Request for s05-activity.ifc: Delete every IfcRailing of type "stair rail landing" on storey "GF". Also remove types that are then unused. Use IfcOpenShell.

First a look at what the model holds.

```python
import ifcopenshell
import ifcopenshell.util.element

model = ifcopenshell.open("s05-activity.ifc")
print(model.schema)
storey = next(s for s in model.by_type("IfcBuildingStorey") if s.Name == "GF")
railings = [e for e in ifcopenshell.util.element.get_decomposition(storey) if e.is_a("IfcRailing")]
seen = {}
for e in railings:
    element_type = ifcopenshell.util.element.get_type(e)
    name = element_type.Name if element_type not in (None, e) else None
    seen[name] = seen.get(name, 0) + 1
for name, count in sorted(seen.items(), key=str):
    print(count, "x", name)
```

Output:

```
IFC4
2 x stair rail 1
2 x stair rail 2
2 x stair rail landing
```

```python
import ifcopenshell
import ifcopenshell.api.root
import ifcopenshell.util.element

model = ifcopenshell.open("s05-activity.ifc")

storey = next(s for s in model.by_type("IfcBuildingStorey") if s.Name == "GF")
railings = [e for e in ifcopenshell.util.element.get_decomposition(storey) if e.is_a("IfcRailing")]
targets = [e for e in railings if (t := ifcopenshell.util.element.get_type(e)) not in (None, e) and t.Name == "stair rail landing"]
types = {ifcopenshell.util.element.get_type(e) for e in targets} - {None, *targets}

for e in targets:
    ifcopenshell.api.root.remove_product(model, product=e)
print(len(targets), "removed")

unused = [t for t in types if not ifcopenshell.util.element.get_types(t)]
for t in unused:
    ifcopenshell.api.root.remove_product(model, product=t)
print(len(unused), "unused types removed")

model.write("s05-activity_edited.ifc")
```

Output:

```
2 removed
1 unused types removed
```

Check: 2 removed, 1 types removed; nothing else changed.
